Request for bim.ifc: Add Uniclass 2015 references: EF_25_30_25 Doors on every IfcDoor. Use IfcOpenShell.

First a look at what the model holds.

```python
import ifcopenshell

model = ifcopenshell.open("bim.ifc")
print(model.schema)
print("classifications:", [c.Name for c in model.by_type("IfcClassification")])
for ifc_class in ("IfcDoor", "IfcRoof", "IfcStair", "IfcWall", "IfcWindow"):
    print(ifc_class, len(model.by_type(ifc_class)))
```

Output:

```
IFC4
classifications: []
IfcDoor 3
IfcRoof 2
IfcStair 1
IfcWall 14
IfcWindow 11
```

```python
import ifcopenshell
import ifcopenshell.api.classification

model = ifcopenshell.open("bim.ifc")

system = ifcopenshell.api.classification.add_classification(model, classification="Uniclass 2015")

codes = {
    "IfcDoor": ("EF_25_30_25", "Doors"),
}
for ifc_class, (code, name) in codes.items():
    products = model.by_type(ifc_class)
    ifcopenshell.api.classification.add_reference(
        model, products=products, classification=system, identification=code, name=name
    )
    print(code, len(products))

model.write("bim_updated.ifc")
```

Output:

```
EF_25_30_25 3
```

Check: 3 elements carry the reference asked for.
